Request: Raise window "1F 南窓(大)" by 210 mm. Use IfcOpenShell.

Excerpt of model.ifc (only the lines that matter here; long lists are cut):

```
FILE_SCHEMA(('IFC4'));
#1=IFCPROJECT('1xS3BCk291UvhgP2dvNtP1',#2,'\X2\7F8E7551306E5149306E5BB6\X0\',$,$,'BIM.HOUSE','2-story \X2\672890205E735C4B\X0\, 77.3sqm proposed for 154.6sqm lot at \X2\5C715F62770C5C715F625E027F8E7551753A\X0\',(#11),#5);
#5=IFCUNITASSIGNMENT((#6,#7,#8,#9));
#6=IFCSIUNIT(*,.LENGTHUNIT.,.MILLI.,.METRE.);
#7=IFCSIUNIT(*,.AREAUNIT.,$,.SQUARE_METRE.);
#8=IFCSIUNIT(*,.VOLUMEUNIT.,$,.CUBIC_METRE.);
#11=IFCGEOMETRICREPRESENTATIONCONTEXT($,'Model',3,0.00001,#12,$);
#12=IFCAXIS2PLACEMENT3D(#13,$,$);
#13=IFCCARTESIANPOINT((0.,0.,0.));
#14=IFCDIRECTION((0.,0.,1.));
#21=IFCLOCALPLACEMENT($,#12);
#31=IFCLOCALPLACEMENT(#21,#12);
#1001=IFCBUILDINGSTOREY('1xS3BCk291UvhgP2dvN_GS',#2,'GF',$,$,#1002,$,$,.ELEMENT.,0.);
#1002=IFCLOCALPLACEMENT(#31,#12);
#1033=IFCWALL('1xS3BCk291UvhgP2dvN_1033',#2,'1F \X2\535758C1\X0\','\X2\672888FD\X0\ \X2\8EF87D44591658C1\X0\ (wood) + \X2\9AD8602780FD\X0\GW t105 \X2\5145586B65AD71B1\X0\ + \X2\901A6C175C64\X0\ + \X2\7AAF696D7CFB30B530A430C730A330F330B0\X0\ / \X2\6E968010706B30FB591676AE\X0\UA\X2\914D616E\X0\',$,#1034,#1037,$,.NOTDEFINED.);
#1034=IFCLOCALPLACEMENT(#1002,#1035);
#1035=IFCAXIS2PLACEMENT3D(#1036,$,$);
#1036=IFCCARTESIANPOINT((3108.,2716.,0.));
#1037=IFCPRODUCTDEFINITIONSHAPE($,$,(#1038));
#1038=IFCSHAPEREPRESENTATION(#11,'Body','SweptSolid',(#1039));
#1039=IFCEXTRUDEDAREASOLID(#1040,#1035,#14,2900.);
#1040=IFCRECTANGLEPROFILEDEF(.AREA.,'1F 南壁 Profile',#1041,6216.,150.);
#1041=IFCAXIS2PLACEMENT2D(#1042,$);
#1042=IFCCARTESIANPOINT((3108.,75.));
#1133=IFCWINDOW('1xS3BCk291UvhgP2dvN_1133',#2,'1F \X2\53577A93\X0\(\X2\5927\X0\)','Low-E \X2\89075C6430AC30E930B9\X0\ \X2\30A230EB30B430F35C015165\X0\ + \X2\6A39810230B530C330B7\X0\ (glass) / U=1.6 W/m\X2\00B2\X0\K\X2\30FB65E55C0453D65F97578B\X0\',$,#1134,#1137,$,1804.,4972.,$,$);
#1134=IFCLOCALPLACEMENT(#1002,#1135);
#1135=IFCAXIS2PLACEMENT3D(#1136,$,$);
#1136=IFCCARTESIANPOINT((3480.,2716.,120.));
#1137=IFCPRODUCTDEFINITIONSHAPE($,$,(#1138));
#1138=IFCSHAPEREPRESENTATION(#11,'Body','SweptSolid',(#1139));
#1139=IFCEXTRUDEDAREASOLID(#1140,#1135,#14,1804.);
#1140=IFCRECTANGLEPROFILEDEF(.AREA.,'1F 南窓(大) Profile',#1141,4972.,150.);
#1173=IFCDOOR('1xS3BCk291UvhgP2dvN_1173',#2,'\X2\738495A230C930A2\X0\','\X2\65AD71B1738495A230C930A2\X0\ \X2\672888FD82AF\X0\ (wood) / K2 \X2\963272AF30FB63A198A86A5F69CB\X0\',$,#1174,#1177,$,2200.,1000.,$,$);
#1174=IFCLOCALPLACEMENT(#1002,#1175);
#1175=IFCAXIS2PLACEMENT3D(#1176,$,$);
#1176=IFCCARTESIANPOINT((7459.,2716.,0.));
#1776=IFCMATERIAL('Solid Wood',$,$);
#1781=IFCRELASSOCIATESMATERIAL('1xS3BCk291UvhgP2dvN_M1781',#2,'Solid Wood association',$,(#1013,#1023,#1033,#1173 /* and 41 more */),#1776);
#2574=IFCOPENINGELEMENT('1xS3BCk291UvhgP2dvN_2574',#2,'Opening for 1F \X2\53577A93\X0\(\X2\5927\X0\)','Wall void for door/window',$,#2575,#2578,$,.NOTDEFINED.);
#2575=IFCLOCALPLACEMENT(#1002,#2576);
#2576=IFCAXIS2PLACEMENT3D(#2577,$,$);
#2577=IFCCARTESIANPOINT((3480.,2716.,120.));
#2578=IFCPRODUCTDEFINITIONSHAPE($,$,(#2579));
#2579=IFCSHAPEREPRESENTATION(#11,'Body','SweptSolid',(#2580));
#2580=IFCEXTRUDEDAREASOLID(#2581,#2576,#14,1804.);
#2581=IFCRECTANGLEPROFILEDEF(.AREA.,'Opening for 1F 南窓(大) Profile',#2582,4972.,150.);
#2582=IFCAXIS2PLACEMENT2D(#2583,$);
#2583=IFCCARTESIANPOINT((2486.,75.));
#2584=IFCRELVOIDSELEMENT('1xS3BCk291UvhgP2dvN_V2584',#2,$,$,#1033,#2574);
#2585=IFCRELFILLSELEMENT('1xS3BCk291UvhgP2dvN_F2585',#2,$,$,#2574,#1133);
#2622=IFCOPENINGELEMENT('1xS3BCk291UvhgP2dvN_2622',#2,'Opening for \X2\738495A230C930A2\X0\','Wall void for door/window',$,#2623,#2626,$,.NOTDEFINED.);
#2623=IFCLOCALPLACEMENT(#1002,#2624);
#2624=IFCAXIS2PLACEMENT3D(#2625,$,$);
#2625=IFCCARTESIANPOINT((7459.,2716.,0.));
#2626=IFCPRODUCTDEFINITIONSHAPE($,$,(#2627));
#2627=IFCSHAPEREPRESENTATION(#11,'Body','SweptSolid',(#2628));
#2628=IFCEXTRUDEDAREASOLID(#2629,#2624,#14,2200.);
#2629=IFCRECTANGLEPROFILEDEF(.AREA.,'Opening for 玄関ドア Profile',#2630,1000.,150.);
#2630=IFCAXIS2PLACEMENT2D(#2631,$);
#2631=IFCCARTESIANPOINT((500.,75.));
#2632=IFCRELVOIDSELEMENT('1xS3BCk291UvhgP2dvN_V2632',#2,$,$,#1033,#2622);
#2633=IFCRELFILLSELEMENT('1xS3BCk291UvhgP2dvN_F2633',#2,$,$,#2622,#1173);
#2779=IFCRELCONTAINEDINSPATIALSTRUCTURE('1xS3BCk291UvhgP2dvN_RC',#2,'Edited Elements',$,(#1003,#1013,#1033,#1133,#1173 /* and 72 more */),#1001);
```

```python
import numpy as np
import ifcopenshell
import ifcopenshell.api.geometry
import ifcopenshell.util.placement
import ifcopenshell.util.unit

model = ifcopenshell.open("model.ifc")
unit_scale = ifcopenshell.util.unit.calculate_unit_scale(model)

window = model.by_id(1133)
opening = window.FillsVoids[0].RelatingOpeningElement
dz = 0.21 / unit_scale

shift = np.array([0.0, 0.0, dz])
# The window is not placed relative to its opening, so move both.
for product in (opening, window):
    matrix = ifcopenshell.util.placement.get_local_placement(product.ObjectPlacement)
    matrix[:3, 3] += shift
    ifcopenshell.api.geometry.edit_object_placement(model, product=product, matrix=matrix, is_si=False)

print(f"moved by {dz * unit_scale:+.3f} m")

model.write("model_updated.ifc")
```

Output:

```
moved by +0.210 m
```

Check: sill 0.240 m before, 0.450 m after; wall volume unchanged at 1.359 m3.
